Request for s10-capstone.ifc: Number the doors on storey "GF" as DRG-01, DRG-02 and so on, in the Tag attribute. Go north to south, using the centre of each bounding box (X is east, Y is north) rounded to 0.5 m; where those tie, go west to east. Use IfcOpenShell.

First a look at what the model holds.

```python
import ifcopenshell
import ifcopenshell.util.element
import ifcopenshell.util.placement

model = ifcopenshell.open("s10-capstone.ifc")
print(model.schema)
storey = next(s for s in model.by_type("IfcBuildingStorey") if s.Name == "GF")
doors = [e for e in ifcopenshell.util.element.get_decomposition(storey) if e.is_a("IfcDoor")]
for e in sorted(doors, key=lambda e: e.id()):
    origin = ifcopenshell.util.placement.get_local_placement(e.ObjectPlacement)[:3, 3]
    print(e.id(), e.Tag, e.Name, origin.round(2) + 0.0, sep=" | ")
```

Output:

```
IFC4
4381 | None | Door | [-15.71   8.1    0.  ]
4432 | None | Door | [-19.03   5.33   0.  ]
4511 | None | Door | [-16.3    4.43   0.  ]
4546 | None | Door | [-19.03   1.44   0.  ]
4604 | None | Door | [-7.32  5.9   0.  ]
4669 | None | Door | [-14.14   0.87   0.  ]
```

```python
import ifcopenshell
import ifcopenshell.geom
import ifcopenshell.util.element
import ifcopenshell.util.shape

model = ifcopenshell.open("s10-capstone.ifc")
settings = ifcopenshell.geom.settings()
settings.set("use-world-coords", True)


def centre(element):
    shape = ifcopenshell.geom.create_shape(settings, element)
    return ifcopenshell.util.shape.get_bbox_centroid(shape.geometry)


storey = next(s for s in model.by_type("IfcBuildingStorey") if s.Name == "GF")
doors = [e for e in ifcopenshell.util.element.get_decomposition(storey) if e.is_a("IfcDoor")]

# Insertion points can sit at a corner or the storey origin, so sort by the geometry (in metres).
centres = {e: centre(e) for e in doors}
doors.sort(key=lambda e: (-round(centres[e][1] / 0.5), centres[e][0]))

for i, e in enumerate(doors, start=1):
    number = f"DRG-{i:02d}"
    e.Tag = number
    print(e.id(), number)

model.write("s10-capstone-out.ifc")
```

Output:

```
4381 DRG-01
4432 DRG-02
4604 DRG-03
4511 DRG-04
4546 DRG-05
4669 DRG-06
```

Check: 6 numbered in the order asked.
